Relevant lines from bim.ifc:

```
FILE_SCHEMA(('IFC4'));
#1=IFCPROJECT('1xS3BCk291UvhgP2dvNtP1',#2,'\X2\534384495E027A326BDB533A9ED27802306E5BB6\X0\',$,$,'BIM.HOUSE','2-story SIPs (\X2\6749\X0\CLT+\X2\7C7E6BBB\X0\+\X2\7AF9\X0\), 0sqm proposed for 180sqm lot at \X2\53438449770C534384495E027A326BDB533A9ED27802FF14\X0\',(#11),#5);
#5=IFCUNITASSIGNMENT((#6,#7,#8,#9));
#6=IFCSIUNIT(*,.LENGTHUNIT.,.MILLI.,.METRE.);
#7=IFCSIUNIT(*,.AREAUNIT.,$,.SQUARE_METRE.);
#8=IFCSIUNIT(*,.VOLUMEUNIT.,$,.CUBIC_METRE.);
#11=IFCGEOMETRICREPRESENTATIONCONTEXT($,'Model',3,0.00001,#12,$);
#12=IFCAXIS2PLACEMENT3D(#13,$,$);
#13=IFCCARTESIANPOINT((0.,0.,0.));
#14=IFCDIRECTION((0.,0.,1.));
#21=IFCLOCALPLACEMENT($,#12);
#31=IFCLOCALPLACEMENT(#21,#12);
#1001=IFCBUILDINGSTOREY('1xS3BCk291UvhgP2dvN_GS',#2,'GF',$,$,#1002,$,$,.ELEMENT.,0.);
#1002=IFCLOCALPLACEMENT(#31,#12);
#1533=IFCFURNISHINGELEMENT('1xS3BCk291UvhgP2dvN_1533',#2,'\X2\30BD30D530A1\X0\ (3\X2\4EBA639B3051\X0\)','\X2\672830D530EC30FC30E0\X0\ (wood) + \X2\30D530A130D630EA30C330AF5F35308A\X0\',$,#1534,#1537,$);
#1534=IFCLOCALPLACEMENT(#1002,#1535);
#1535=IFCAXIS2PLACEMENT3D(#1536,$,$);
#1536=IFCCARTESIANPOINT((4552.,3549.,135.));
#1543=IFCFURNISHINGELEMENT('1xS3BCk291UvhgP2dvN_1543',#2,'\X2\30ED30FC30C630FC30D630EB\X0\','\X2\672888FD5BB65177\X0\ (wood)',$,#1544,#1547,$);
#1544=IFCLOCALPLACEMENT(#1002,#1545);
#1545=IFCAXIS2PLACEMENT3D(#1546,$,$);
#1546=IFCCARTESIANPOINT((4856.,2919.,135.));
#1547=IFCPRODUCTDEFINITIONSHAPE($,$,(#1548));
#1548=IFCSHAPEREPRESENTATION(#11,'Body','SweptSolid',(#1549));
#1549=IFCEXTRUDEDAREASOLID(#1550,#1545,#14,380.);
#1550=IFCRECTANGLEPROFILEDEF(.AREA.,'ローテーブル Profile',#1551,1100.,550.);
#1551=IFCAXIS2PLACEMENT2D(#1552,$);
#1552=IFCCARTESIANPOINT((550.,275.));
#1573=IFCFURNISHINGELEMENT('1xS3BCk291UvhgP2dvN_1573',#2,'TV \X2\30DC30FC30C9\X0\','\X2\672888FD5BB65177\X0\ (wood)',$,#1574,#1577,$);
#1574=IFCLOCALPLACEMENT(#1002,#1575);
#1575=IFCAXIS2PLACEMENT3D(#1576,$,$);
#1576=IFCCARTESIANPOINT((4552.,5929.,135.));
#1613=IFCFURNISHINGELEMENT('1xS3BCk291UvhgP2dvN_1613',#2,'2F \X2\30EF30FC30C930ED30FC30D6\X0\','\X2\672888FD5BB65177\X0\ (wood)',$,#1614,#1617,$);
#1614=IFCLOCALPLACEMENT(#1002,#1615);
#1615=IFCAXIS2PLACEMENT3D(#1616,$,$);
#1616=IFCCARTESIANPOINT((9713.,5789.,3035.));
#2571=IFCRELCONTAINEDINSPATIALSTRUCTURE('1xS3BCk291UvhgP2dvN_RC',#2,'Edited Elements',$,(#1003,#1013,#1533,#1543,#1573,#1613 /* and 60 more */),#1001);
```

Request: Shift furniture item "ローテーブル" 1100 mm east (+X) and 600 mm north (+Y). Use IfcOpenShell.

```python
import ifcopenshell
import ifcopenshell.api.geometry
import ifcopenshell.util.placement
import ifcopenshell.util.unit

model = ifcopenshell.open("bim.ifc")
unit_scale = ifcopenshell.util.unit.calculate_unit_scale(model)

item = model.by_guid("1xS3BCk291UvhgP2dvN_1543")
matrix = ifcopenshell.util.placement.get_local_placement(item.ObjectPlacement)
matrix[0, 3] += 1.1 / unit_scale
matrix[1, 3] += 0.6 / unit_scale
ifcopenshell.api.geometry.edit_object_placement(model, product=item, matrix=matrix, is_si=False)

print(ifcopenshell.util.placement.get_local_placement(item.ObjectPlacement).round(3) + 0.0)

model.write("bim_edited.ifc")
```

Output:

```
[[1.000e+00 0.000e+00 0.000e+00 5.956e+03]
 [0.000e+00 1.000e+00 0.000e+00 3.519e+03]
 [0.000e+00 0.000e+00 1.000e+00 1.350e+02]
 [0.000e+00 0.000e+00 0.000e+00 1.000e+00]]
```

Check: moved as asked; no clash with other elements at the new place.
